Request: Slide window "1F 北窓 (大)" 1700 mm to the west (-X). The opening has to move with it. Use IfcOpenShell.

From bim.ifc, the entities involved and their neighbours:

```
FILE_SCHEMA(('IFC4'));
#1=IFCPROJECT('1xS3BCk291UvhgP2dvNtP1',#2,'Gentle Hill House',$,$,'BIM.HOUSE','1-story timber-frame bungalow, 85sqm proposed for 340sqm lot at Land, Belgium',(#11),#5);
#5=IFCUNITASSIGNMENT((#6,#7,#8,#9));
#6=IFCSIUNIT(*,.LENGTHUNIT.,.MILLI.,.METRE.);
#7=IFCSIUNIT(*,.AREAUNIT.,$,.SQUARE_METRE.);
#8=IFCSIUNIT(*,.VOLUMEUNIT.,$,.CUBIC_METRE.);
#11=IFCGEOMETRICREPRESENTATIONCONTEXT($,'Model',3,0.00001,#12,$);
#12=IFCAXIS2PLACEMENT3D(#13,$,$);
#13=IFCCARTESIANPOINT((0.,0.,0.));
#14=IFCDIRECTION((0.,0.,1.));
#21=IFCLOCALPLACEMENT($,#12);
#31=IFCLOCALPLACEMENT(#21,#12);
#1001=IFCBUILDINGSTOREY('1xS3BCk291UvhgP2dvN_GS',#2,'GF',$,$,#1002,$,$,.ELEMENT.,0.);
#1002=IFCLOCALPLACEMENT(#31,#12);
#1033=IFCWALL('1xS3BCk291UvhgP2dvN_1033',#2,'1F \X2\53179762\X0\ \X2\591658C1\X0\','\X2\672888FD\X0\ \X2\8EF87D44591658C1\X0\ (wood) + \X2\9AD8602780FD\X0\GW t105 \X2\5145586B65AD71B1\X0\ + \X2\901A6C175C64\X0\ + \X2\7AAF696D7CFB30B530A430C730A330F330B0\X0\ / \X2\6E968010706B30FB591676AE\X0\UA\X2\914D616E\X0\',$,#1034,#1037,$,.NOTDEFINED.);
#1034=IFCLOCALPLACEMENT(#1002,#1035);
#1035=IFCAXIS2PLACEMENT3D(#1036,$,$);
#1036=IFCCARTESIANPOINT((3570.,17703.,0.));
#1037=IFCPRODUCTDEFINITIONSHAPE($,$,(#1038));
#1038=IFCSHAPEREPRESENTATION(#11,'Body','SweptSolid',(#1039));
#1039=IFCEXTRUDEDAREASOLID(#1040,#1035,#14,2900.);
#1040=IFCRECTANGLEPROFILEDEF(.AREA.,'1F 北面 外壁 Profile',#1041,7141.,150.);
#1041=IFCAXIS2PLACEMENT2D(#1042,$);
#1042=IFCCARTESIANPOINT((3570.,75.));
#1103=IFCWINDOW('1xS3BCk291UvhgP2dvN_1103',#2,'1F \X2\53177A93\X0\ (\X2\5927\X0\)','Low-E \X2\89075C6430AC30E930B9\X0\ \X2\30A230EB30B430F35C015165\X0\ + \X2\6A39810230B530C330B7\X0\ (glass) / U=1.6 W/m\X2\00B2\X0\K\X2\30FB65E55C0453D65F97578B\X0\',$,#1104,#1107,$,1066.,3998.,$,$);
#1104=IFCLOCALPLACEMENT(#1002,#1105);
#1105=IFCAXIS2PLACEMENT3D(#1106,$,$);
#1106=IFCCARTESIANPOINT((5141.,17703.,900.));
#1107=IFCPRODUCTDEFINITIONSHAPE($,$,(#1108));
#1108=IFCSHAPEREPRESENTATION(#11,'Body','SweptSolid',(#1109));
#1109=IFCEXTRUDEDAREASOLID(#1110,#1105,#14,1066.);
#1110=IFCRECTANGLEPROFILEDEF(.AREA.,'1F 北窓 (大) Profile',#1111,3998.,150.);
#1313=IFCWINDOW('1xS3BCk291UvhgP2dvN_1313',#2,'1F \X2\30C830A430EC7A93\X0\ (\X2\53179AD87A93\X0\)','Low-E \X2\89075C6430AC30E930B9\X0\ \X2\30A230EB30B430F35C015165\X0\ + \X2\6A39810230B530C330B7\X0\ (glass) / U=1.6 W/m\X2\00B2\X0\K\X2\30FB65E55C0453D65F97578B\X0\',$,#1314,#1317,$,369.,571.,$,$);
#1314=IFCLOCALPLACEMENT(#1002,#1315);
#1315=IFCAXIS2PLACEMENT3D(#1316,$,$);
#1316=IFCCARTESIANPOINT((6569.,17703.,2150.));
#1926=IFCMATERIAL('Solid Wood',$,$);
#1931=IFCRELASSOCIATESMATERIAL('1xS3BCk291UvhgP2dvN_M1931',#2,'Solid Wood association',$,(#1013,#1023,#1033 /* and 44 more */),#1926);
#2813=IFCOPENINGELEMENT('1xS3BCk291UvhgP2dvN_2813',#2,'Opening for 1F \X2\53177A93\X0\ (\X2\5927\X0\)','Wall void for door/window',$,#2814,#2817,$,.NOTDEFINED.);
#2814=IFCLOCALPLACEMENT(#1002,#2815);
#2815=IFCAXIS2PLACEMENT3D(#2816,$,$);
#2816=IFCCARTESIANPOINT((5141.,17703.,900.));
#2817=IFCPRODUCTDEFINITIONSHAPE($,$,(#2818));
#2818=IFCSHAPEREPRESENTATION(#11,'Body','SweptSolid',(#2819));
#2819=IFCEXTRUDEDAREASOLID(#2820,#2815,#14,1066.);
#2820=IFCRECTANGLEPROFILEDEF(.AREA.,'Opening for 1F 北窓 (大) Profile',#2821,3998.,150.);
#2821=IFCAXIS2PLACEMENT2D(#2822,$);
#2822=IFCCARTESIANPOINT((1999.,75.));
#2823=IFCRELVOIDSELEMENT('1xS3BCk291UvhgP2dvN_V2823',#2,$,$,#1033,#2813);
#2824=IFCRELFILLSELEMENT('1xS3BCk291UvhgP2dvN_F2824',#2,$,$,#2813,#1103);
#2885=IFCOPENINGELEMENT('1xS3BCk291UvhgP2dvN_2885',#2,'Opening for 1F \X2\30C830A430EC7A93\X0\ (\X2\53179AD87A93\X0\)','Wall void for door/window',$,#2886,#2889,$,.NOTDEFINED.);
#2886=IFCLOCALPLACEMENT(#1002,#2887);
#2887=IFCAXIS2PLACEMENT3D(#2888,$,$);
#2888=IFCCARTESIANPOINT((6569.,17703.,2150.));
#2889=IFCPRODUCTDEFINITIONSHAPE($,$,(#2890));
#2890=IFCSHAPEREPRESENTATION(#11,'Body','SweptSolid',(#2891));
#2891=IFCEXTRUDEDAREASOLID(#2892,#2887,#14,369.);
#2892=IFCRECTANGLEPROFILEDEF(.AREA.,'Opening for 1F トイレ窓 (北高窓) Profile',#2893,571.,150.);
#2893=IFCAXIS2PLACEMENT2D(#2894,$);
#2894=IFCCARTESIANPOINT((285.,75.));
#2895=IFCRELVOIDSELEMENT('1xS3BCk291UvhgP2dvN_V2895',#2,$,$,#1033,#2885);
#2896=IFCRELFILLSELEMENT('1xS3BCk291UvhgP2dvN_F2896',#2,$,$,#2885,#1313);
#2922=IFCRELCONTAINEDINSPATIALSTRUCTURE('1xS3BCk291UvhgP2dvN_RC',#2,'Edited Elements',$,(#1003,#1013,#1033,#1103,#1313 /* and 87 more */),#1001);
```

```python
import ifcopenshell
import ifcopenshell.api.geometry
import ifcopenshell.util.placement
import ifcopenshell.util.unit

model = ifcopenshell.open("bim.ifc")
unit_scale = ifcopenshell.util.unit.calculate_unit_scale(model)

window = model.by_id(1103)
opening = window.FillsVoids[0].RelatingOpeningElement
wall = opening.VoidsElements[0].RelatingBuildingElement

wall_matrix = ifcopenshell.util.placement.get_local_placement(wall.ObjectPlacement)
shift = wall_matrix[:3, 0] * -1.7 / unit_scale
before = ifcopenshell.util.placement.get_local_placement(window.ObjectPlacement)[:3, 3].copy()

# The window is not placed relative to its opening, so move both.
for product in (opening, window):
    matrix = ifcopenshell.util.placement.get_local_placement(product.ObjectPlacement)
    matrix[:3, 3] += shift
    ifcopenshell.api.geometry.edit_object_placement(model, product=product, matrix=matrix, is_si=False)

after = ifcopenshell.util.placement.get_local_placement(window.ObjectPlacement)[:3, 3]
print("window moved by", (after - before).round(3) + 0.0)

model.write("bim_edited.ifc")
```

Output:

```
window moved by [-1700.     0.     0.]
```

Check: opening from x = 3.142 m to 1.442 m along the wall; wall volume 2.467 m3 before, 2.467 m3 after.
